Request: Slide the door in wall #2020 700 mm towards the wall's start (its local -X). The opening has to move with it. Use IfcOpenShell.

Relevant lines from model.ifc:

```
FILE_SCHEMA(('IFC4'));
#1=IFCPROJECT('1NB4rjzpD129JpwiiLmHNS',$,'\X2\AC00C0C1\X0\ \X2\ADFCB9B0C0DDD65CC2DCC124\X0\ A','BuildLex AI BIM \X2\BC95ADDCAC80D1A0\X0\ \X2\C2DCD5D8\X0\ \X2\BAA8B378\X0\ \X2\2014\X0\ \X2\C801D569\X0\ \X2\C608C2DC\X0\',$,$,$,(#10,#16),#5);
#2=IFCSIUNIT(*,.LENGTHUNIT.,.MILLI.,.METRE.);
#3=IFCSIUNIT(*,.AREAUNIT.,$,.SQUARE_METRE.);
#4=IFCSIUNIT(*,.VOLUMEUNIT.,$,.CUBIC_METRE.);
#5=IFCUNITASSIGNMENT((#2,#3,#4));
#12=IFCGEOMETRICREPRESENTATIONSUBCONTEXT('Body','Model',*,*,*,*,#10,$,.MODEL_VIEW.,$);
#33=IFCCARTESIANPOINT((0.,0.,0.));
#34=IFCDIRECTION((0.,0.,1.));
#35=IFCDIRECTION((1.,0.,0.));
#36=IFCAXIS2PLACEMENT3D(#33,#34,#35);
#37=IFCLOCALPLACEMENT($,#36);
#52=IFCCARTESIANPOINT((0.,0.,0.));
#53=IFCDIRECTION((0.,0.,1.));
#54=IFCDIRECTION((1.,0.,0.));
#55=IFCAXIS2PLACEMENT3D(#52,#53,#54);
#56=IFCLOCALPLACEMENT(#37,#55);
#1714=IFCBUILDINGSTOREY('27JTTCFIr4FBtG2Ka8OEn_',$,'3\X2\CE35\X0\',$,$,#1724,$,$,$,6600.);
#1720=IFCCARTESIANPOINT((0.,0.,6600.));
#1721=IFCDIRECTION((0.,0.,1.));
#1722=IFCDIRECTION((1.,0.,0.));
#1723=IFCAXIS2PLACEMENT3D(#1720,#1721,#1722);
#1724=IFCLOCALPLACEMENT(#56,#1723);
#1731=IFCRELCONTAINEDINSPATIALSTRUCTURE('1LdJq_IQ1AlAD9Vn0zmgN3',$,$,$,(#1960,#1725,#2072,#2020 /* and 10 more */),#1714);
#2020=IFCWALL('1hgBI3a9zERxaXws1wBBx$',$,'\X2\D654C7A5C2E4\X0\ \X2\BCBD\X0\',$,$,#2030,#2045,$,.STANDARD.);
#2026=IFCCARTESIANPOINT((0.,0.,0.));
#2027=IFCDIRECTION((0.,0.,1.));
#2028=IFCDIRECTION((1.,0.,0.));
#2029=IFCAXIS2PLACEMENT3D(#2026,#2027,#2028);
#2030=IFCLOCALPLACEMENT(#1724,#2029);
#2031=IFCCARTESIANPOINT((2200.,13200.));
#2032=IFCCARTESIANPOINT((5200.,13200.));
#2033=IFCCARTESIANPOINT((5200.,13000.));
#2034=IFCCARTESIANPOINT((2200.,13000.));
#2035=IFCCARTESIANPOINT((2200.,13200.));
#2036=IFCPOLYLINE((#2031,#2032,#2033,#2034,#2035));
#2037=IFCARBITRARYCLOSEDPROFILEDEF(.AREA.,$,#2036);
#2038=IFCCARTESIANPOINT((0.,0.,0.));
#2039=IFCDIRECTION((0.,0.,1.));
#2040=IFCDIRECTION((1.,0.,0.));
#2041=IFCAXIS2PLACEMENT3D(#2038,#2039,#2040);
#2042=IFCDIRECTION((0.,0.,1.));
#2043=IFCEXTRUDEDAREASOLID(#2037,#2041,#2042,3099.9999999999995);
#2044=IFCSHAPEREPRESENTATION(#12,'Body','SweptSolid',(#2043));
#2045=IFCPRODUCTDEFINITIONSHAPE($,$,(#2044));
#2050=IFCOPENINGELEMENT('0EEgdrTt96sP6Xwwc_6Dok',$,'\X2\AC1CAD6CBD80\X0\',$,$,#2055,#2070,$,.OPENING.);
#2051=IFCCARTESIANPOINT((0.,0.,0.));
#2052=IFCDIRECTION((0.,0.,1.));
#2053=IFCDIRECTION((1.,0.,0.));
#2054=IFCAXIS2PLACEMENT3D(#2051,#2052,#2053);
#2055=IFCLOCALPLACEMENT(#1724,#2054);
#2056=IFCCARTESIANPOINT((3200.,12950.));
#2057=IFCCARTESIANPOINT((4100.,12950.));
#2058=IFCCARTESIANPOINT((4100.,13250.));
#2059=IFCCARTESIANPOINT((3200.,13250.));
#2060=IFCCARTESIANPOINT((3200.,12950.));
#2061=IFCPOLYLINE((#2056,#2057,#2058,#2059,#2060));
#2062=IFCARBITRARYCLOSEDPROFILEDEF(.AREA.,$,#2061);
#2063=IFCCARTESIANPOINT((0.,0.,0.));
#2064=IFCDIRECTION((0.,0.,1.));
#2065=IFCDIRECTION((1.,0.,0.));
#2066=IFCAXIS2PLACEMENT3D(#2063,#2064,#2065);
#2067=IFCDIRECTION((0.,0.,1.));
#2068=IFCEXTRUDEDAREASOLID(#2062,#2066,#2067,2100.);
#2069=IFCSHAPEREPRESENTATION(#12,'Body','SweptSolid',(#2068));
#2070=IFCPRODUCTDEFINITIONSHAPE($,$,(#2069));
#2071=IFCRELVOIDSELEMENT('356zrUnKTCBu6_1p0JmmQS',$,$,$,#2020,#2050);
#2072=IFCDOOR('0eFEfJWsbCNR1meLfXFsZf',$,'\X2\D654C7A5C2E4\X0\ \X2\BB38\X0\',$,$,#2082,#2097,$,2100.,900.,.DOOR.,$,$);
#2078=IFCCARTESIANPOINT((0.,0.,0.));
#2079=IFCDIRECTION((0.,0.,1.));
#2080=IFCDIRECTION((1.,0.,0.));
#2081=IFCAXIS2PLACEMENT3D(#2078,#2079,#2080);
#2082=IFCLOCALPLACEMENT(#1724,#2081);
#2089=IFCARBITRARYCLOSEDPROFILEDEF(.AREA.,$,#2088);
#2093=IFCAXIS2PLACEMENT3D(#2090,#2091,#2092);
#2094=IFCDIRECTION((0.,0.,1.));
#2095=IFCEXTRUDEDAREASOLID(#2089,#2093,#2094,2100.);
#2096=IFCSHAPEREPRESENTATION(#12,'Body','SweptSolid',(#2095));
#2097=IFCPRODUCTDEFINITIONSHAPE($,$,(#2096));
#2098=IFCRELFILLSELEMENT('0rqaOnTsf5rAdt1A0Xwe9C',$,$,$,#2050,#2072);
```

```python
import ifcopenshell
import ifcopenshell.api.geometry
import ifcopenshell.util.placement

model = ifcopenshell.open("model.ifc")

door = model.by_id(2072)
opening = door.FillsVoids[0].RelatingOpeningElement
wall = opening.VoidsElements[0].RelatingBuildingElement

wall_matrix = ifcopenshell.util.placement.get_local_placement(wall.ObjectPlacement)
shift = wall_matrix[:3, 0] * -700.0
before = ifcopenshell.util.placement.get_local_placement(door.ObjectPlacement)[:3, 3].copy()

# The door is not placed relative to its opening, so move both.
for product in (opening, door):
    matrix = ifcopenshell.util.placement.get_local_placement(product.ObjectPlacement)
    matrix[:3, 3] += shift
    ifcopenshell.api.geometry.edit_object_placement(model, product=product, matrix=matrix, is_si=False)

after = ifcopenshell.util.placement.get_local_placement(door.ObjectPlacement)[:3, 3]
print("door moved by", (after - before).round(3) + 0.0)

model.write("model_edited.ifc")
```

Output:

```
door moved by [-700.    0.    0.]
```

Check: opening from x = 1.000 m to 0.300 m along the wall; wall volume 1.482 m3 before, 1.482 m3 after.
